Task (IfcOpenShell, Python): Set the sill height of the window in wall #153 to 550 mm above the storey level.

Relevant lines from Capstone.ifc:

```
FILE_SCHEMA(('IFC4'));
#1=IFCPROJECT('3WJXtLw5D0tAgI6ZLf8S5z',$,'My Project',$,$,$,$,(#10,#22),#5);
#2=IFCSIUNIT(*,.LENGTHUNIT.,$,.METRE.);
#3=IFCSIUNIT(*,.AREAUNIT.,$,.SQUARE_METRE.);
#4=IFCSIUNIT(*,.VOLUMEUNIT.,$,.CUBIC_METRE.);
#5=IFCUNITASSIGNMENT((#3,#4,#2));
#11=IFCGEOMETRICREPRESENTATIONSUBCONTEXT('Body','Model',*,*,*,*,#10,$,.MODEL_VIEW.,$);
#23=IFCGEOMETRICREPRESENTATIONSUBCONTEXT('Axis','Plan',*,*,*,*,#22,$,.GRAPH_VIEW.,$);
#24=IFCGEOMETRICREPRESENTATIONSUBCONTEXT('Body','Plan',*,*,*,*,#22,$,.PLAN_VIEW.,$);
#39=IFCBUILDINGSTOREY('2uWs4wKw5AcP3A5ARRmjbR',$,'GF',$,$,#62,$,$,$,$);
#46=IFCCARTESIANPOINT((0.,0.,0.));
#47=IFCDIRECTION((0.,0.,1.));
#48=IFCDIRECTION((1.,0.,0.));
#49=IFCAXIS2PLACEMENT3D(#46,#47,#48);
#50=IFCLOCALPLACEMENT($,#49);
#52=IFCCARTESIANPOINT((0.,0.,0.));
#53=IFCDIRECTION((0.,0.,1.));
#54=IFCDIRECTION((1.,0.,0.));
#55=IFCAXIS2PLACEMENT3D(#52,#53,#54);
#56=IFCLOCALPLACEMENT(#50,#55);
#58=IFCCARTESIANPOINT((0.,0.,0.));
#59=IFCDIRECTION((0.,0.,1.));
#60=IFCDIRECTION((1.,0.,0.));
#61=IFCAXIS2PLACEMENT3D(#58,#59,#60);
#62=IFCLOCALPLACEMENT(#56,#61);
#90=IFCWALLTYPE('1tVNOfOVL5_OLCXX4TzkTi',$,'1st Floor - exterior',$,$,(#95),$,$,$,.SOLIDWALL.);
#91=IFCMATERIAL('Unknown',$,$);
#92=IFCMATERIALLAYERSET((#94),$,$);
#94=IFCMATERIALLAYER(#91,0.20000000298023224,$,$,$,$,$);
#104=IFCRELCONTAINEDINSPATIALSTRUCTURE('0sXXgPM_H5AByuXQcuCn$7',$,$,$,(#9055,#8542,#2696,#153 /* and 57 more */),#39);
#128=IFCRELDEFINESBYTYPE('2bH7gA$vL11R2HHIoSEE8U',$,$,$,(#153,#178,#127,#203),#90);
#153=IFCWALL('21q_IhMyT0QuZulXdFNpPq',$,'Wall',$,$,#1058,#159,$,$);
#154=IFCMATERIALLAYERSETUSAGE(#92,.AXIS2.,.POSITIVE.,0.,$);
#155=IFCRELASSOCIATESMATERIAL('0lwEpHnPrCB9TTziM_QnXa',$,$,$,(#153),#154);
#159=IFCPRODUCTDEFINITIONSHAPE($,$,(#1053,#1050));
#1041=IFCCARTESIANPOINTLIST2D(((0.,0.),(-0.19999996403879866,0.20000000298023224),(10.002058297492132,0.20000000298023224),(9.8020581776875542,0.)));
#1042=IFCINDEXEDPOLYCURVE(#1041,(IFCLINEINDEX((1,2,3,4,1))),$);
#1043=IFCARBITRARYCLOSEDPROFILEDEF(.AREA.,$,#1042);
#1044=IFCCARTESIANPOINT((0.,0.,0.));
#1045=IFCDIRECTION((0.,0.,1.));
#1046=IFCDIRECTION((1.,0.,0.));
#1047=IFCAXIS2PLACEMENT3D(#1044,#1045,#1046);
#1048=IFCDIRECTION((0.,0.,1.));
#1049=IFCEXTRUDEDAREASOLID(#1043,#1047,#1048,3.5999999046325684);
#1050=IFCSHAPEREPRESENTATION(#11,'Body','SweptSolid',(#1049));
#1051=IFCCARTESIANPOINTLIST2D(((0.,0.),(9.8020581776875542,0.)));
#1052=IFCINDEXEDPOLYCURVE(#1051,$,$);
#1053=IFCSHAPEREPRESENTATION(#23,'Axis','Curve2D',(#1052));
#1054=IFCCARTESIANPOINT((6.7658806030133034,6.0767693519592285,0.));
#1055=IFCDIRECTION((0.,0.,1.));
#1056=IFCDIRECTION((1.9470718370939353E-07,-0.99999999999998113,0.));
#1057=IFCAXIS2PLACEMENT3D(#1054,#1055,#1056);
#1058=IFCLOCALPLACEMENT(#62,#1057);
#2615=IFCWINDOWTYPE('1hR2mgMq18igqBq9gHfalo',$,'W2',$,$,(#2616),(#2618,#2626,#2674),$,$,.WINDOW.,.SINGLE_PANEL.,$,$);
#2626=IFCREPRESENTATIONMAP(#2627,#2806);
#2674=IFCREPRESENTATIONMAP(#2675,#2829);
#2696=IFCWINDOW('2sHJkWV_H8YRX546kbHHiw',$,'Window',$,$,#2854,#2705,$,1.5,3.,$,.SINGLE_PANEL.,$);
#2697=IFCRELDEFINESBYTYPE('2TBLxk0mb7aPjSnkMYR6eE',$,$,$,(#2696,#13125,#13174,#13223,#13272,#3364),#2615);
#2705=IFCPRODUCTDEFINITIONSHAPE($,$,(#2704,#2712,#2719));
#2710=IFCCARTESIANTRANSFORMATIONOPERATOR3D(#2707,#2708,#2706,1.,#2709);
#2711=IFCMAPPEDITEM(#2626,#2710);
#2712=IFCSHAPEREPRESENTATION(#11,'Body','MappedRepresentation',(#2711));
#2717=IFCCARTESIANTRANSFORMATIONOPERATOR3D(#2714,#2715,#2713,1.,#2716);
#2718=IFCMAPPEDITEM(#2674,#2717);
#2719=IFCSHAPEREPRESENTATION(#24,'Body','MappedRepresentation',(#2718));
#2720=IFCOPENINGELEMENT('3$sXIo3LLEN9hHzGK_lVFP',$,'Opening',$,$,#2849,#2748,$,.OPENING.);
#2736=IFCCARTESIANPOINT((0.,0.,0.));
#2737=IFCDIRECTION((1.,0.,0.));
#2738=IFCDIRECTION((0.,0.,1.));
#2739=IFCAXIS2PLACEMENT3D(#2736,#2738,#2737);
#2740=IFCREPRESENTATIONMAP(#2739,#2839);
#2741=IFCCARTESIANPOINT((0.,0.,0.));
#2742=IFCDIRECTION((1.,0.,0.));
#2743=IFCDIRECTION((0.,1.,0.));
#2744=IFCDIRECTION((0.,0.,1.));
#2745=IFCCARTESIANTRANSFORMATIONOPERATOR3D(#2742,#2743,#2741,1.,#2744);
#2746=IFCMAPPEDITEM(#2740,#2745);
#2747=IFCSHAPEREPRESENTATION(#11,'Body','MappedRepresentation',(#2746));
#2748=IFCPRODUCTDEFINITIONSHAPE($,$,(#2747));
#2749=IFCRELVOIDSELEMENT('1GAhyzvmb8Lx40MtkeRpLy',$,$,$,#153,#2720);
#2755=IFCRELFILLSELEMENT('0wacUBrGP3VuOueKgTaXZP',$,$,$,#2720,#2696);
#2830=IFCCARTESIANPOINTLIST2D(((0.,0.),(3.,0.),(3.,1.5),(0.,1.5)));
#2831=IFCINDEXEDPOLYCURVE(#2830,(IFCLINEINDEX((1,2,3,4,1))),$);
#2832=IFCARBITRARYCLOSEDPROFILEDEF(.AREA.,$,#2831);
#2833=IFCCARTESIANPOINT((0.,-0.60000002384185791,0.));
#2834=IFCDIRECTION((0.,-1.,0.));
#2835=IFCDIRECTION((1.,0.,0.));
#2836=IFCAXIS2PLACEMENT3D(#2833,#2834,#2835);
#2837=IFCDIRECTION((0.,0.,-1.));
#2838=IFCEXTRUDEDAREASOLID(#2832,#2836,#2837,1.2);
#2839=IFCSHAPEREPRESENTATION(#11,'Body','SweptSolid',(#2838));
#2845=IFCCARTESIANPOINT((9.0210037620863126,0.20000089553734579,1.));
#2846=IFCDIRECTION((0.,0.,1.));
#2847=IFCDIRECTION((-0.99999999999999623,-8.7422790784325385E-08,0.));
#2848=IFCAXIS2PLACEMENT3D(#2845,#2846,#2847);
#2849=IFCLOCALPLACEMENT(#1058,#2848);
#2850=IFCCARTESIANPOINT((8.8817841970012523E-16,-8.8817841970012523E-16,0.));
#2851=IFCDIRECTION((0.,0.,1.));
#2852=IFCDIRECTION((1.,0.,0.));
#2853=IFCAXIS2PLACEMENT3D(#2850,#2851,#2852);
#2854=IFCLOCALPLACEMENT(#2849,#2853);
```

```python
import numpy as np
import ifcopenshell
import ifcopenshell.api.geometry
import ifcopenshell.geom
import ifcopenshell.util.element
import ifcopenshell.util.placement
import ifcopenshell.util.shape
import ifcopenshell.util.unit

model = ifcopenshell.open("Capstone.ifc")
unit_scale = ifcopenshell.util.unit.calculate_unit_scale(model)

window = model.by_id(2696)
opening = window.FillsVoids[0].RelatingOpeningElement
storey = ifcopenshell.util.element.get_container(window, ifc_class="IfcBuildingStorey")
level = ifcopenshell.util.placement.get_local_placement(storey.ObjectPlacement)[2, 3]

# The opening's origin need not be at the sill, so measure its lowest point.
shape = ifcopenshell.geom.create_shape(ifcopenshell.geom.settings(), opening)
bottom = ifcopenshell.util.shape.get_shape_bottom_elevation(shape, shape.geometry) / unit_scale
dz = level + 0.55 / unit_scale - bottom

shift = np.array([0.0, 0.0, dz])
# The window is placed relative to its opening, so it follows when the opening moves.
matrix = ifcopenshell.util.placement.get_local_placement(opening.ObjectPlacement)
matrix[:3, 3] += shift
ifcopenshell.api.geometry.edit_object_placement(
    model, product=opening, matrix=matrix, is_si=False, should_transform_children=True
)

print(f"moved by {dz * unit_scale:+.3f} m")

model.write("Capstone_v2.ifc")
```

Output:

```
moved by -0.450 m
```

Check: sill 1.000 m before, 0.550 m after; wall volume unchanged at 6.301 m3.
